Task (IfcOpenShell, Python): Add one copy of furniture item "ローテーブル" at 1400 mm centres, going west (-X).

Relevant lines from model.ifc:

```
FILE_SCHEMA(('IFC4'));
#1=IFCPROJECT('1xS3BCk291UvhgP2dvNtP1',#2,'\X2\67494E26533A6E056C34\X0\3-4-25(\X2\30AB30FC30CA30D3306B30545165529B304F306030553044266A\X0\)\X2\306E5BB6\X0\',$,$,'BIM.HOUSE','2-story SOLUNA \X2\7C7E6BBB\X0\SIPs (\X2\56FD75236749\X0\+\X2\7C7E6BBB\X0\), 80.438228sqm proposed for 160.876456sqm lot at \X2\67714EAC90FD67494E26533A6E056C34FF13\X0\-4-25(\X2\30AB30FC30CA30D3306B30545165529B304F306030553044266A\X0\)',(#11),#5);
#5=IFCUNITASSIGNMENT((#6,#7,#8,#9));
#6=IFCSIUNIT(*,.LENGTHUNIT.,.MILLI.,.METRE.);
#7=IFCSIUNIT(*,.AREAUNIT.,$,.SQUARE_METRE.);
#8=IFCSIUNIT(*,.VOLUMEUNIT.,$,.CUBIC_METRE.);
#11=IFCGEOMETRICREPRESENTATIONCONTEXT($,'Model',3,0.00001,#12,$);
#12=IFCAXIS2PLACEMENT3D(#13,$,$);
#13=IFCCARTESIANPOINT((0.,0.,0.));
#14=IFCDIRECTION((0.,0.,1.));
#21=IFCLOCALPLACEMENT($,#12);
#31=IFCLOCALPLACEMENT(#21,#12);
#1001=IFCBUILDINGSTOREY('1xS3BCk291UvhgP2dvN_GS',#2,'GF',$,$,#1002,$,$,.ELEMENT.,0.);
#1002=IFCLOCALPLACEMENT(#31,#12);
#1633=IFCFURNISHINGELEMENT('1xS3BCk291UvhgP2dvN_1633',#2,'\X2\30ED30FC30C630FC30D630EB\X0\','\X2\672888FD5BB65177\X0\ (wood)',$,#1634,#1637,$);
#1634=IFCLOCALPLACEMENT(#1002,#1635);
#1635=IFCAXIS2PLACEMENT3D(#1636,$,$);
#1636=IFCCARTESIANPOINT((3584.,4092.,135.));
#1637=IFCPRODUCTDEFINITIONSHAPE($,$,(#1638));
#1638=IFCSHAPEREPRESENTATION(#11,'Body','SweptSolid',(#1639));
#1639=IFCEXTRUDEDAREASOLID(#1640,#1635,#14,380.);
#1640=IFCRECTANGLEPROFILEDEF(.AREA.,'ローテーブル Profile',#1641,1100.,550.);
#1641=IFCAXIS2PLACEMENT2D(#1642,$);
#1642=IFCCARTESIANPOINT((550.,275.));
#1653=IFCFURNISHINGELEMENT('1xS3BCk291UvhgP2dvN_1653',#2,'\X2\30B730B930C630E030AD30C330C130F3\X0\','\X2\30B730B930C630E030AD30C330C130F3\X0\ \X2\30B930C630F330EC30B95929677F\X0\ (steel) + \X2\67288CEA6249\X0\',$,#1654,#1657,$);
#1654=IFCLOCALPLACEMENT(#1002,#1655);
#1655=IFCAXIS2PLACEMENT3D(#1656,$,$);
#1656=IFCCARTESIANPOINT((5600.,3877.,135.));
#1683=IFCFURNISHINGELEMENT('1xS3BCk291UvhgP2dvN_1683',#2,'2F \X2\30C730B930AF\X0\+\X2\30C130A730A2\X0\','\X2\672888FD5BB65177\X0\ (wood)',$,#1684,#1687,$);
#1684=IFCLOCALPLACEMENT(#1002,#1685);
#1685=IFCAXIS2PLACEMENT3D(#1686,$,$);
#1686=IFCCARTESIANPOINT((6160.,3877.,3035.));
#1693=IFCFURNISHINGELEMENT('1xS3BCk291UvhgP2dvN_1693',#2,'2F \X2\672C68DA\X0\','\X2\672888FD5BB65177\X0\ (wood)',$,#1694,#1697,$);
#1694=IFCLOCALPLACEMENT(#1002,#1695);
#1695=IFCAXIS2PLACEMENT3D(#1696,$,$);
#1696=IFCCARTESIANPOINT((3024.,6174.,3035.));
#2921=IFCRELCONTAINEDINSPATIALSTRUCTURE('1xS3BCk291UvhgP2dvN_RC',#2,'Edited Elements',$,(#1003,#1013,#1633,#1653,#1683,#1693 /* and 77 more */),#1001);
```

```python
import numpy as np
import ifcopenshell
import ifcopenshell.api.geometry
import ifcopenshell.api.root
import ifcopenshell.util.element
import ifcopenshell.util.placement

model = ifcopenshell.open("model.ifc")


def reuse_history(source, copy):
    """copy_class also copies each property set's owner history, people and application; keep the originals."""
    for rel in copy.IsDefinedBy:
        if rel.is_a("IfcRelDefinesByProperties") and (history := rel.RelatingPropertyDefinition.OwnerHistory):
            rel.RelatingPropertyDefinition.OwnerHistory = source.OwnerHistory
            ifcopenshell.util.element.remove_deep2(model, history)


source = model.by_id(1633)
base = ifcopenshell.util.placement.get_local_placement(source.ObjectPlacement)
step = np.array([-1.0, 0.0, 0.0]) * 1400.0

for i in range(1, 2):
    copy = ifcopenshell.api.root.copy_class(model, product=source)
    copy.Representation = ifcopenshell.util.element.copy_deep(
        model, source.Representation, exclude=["IfcGeometricRepresentationContext", "IfcRepresentationMap"]
    )
    reuse_history(source, copy)
    matrix = base.copy()
    matrix[:3, 3] += i * step
    print("added at", matrix[:3, 3].round(3) + 0.0)
    ifcopenshell.api.geometry.edit_object_placement(model, product=copy, matrix=matrix, is_si=False)

model.write("model-out.ifc")
```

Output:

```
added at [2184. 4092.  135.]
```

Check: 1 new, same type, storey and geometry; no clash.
